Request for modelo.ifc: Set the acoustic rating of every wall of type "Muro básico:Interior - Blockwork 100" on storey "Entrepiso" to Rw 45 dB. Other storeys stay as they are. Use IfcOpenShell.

First a look at what the model holds.

```python
import ifcopenshell
import ifcopenshell.util.element

model = ifcopenshell.open("modelo.ifc")
print(model.schema)
storey = next(s for s in model.by_type("IfcBuildingStorey") if s.Name == "Entrepiso")
walls = [e for e in ifcopenshell.util.element.get_decomposition(storey) if e.is_a("IfcWall")]
seen = {}
for e in walls:
    element_type = ifcopenshell.util.element.get_type(e)
    key = (element_type.Name if element_type != e and element_type else None, ifcopenshell.util.element.get_pset(e, "Pset_WallCommon", "AcousticRating"))
    seen[key] = seen.get(key, 0) + 1
for (name, value), count in sorted(seen.items(), key=str):
    print(count, "x", name, "|", value)
```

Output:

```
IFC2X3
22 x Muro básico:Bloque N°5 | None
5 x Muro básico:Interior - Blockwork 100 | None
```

```python
import ifcopenshell
import ifcopenshell.api.pset
import ifcopenshell.util.element

model = ifcopenshell.open("modelo.ifc")

storey = next(s for s in model.by_type("IfcBuildingStorey") if s.Name == "Entrepiso")
walls = [e for e in ifcopenshell.util.element.get_decomposition(storey) if e.is_a("IfcWall")]

count = 0
for e in walls:
    element_type = ifcopenshell.util.element.get_type(e)
    if element_type in (None, e) or element_type.Name != "Muro básico:Interior - Blockwork 100":
        continue
    # add_pset returns the element's existing set when there is one.
    pset = ifcopenshell.api.pset.add_pset(model, product=e, name="Pset_WallCommon")
    ifcopenshell.api.pset.edit_pset(model, pset=pset, properties={"AcousticRating": "Rw 45 dB"})
    count += 1

print(count, "walls updated")

model.write("modelo-out.ifc")
```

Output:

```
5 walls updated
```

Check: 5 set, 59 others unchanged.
